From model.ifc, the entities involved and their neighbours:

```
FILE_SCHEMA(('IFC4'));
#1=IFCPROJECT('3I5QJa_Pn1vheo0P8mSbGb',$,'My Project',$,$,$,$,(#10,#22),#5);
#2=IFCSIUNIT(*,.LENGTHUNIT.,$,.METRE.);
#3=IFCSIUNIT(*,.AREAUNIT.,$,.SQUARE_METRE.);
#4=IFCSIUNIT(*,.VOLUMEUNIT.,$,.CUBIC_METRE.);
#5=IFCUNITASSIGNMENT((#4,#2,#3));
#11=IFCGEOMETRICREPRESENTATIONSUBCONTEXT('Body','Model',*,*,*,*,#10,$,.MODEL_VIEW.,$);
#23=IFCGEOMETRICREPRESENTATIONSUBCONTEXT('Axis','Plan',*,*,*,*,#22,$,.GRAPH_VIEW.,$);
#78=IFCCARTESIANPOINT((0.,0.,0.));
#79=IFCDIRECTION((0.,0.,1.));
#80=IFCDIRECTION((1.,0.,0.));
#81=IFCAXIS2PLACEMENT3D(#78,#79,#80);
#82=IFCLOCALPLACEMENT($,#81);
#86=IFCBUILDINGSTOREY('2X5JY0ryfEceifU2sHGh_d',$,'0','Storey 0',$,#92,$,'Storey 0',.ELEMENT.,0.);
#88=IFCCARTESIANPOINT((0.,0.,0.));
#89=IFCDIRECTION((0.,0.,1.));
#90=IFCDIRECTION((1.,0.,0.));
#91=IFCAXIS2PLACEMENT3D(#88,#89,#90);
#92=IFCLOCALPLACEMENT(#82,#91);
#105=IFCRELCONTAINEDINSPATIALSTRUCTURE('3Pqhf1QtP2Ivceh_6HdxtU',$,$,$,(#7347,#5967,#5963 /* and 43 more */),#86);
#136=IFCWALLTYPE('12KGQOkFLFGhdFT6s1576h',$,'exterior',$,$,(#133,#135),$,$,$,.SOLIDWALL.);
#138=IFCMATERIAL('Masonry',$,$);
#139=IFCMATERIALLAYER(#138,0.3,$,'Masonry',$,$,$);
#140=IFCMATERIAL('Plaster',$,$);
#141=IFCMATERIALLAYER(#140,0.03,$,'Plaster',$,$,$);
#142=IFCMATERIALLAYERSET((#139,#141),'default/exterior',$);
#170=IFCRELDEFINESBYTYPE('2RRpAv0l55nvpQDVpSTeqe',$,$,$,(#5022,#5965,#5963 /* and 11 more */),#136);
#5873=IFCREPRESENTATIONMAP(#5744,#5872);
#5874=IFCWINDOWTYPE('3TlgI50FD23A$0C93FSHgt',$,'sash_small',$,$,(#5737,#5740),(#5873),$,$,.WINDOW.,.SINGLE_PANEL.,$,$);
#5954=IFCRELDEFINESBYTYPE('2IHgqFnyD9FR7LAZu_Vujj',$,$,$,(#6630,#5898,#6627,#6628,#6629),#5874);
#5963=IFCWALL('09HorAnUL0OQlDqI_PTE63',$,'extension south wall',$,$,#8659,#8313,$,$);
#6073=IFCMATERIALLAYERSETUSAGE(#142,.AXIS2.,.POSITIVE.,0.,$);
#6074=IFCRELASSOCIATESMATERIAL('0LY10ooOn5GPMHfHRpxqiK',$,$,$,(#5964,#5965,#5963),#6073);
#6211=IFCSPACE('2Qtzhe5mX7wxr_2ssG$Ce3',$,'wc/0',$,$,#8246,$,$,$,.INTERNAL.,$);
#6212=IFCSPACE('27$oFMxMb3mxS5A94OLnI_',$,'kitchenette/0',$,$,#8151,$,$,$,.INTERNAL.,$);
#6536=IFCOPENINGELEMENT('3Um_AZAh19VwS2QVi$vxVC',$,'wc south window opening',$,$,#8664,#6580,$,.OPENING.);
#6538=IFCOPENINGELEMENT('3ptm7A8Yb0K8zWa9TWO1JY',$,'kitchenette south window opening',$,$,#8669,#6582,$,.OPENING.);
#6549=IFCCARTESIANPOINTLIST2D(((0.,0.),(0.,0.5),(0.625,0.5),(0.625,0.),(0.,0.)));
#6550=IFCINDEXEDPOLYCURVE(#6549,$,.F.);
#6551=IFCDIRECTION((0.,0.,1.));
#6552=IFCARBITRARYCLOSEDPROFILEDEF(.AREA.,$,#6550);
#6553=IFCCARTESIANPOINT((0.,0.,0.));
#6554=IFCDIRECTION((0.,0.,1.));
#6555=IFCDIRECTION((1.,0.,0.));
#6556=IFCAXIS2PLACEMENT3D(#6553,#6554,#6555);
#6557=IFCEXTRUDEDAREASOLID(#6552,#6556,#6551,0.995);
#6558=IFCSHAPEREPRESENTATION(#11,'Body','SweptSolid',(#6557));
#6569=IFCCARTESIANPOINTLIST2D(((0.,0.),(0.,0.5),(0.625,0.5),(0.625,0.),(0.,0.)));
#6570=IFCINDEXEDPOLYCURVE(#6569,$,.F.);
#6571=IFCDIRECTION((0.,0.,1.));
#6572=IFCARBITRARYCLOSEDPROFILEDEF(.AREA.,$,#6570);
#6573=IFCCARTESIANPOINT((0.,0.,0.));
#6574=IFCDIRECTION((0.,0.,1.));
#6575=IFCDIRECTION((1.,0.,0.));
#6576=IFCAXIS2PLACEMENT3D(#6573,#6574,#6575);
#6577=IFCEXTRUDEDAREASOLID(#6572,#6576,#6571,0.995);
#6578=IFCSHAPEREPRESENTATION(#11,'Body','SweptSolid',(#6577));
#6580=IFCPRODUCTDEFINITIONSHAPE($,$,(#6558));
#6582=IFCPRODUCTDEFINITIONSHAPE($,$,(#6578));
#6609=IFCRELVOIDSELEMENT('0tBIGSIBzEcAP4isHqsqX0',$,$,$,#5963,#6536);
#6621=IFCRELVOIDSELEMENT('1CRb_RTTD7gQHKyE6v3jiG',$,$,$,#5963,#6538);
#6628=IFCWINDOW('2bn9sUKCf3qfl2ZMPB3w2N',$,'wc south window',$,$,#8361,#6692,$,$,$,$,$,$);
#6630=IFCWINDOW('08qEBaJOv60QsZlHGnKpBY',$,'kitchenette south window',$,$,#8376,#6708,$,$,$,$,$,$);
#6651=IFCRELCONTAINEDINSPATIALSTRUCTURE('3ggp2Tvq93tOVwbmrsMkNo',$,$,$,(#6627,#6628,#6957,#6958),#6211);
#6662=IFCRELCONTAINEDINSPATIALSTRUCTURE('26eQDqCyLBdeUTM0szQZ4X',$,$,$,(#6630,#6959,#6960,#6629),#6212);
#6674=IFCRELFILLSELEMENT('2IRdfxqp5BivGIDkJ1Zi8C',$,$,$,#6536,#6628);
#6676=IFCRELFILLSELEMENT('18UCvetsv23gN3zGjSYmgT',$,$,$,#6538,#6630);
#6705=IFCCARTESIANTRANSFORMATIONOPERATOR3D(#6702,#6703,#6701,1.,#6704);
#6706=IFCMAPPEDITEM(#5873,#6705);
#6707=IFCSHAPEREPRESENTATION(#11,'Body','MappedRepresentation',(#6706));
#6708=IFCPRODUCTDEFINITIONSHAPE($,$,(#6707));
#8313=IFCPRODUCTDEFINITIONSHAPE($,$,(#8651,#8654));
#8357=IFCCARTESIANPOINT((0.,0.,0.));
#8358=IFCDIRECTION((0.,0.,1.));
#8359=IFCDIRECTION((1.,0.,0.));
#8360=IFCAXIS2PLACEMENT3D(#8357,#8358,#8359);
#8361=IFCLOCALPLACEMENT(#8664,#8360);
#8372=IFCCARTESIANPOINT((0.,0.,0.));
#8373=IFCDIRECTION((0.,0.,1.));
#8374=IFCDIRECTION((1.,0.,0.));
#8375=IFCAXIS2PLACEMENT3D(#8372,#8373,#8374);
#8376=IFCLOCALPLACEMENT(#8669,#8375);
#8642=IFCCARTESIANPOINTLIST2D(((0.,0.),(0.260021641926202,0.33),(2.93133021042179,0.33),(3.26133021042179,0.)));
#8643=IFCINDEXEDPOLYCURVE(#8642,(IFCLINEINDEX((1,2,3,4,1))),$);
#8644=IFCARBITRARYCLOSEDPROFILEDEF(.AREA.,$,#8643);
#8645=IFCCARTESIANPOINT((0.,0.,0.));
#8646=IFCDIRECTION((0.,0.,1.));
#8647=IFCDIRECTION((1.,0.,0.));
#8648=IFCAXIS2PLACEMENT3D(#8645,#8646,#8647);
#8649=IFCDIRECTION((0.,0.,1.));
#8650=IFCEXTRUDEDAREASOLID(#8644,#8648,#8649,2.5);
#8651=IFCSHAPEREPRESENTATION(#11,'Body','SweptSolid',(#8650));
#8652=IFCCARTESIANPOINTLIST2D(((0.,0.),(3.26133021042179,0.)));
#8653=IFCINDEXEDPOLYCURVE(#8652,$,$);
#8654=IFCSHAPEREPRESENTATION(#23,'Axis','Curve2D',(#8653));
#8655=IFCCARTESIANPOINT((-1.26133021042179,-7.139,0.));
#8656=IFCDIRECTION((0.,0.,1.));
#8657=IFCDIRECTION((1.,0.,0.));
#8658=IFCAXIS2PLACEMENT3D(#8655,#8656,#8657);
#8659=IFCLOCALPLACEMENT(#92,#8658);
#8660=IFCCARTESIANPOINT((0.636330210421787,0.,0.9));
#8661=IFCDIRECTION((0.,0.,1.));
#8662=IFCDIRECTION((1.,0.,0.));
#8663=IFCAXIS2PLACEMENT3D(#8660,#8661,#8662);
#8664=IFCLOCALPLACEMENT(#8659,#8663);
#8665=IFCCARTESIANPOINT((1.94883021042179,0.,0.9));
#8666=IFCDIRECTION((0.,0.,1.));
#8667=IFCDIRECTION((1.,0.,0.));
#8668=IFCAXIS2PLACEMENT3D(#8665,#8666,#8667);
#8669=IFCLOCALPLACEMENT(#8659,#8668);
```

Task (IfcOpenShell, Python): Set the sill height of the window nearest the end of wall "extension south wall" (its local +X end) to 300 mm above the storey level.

```python
import numpy as np
import ifcopenshell
import ifcopenshell.api.geometry
import ifcopenshell.geom
import ifcopenshell.util.element
import ifcopenshell.util.placement
import ifcopenshell.util.shape
import ifcopenshell.util.unit

model = ifcopenshell.open("model.ifc")
unit_scale = ifcopenshell.util.unit.calculate_unit_scale(model)

window = model.by_guid("08qEBaJOv60QsZlHGnKpBY")
opening = window.FillsVoids[0].RelatingOpeningElement
storey = ifcopenshell.util.element.get_container(window, ifc_class="IfcBuildingStorey")
level = ifcopenshell.util.placement.get_local_placement(storey.ObjectPlacement)[2, 3]

# The opening's origin need not be at the sill, so measure its lowest point.
shape = ifcopenshell.geom.create_shape(ifcopenshell.geom.settings(), opening)
bottom = ifcopenshell.util.shape.get_shape_bottom_elevation(shape, shape.geometry) / unit_scale
dz = level + 0.3 / unit_scale - bottom

shift = np.array([0.0, 0.0, dz])
# The window is placed relative to its opening, so it follows when the opening moves.
matrix = ifcopenshell.util.placement.get_local_placement(opening.ObjectPlacement)
matrix[:3, 3] += shift
ifcopenshell.api.geometry.edit_object_placement(
    model, product=opening, matrix=matrix, is_si=False, should_transform_children=True
)

print(f"moved by {dz * unit_scale:+.3f} m")

model.write("model_edited.ifc")
```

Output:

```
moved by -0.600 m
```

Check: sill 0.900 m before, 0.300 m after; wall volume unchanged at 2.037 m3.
